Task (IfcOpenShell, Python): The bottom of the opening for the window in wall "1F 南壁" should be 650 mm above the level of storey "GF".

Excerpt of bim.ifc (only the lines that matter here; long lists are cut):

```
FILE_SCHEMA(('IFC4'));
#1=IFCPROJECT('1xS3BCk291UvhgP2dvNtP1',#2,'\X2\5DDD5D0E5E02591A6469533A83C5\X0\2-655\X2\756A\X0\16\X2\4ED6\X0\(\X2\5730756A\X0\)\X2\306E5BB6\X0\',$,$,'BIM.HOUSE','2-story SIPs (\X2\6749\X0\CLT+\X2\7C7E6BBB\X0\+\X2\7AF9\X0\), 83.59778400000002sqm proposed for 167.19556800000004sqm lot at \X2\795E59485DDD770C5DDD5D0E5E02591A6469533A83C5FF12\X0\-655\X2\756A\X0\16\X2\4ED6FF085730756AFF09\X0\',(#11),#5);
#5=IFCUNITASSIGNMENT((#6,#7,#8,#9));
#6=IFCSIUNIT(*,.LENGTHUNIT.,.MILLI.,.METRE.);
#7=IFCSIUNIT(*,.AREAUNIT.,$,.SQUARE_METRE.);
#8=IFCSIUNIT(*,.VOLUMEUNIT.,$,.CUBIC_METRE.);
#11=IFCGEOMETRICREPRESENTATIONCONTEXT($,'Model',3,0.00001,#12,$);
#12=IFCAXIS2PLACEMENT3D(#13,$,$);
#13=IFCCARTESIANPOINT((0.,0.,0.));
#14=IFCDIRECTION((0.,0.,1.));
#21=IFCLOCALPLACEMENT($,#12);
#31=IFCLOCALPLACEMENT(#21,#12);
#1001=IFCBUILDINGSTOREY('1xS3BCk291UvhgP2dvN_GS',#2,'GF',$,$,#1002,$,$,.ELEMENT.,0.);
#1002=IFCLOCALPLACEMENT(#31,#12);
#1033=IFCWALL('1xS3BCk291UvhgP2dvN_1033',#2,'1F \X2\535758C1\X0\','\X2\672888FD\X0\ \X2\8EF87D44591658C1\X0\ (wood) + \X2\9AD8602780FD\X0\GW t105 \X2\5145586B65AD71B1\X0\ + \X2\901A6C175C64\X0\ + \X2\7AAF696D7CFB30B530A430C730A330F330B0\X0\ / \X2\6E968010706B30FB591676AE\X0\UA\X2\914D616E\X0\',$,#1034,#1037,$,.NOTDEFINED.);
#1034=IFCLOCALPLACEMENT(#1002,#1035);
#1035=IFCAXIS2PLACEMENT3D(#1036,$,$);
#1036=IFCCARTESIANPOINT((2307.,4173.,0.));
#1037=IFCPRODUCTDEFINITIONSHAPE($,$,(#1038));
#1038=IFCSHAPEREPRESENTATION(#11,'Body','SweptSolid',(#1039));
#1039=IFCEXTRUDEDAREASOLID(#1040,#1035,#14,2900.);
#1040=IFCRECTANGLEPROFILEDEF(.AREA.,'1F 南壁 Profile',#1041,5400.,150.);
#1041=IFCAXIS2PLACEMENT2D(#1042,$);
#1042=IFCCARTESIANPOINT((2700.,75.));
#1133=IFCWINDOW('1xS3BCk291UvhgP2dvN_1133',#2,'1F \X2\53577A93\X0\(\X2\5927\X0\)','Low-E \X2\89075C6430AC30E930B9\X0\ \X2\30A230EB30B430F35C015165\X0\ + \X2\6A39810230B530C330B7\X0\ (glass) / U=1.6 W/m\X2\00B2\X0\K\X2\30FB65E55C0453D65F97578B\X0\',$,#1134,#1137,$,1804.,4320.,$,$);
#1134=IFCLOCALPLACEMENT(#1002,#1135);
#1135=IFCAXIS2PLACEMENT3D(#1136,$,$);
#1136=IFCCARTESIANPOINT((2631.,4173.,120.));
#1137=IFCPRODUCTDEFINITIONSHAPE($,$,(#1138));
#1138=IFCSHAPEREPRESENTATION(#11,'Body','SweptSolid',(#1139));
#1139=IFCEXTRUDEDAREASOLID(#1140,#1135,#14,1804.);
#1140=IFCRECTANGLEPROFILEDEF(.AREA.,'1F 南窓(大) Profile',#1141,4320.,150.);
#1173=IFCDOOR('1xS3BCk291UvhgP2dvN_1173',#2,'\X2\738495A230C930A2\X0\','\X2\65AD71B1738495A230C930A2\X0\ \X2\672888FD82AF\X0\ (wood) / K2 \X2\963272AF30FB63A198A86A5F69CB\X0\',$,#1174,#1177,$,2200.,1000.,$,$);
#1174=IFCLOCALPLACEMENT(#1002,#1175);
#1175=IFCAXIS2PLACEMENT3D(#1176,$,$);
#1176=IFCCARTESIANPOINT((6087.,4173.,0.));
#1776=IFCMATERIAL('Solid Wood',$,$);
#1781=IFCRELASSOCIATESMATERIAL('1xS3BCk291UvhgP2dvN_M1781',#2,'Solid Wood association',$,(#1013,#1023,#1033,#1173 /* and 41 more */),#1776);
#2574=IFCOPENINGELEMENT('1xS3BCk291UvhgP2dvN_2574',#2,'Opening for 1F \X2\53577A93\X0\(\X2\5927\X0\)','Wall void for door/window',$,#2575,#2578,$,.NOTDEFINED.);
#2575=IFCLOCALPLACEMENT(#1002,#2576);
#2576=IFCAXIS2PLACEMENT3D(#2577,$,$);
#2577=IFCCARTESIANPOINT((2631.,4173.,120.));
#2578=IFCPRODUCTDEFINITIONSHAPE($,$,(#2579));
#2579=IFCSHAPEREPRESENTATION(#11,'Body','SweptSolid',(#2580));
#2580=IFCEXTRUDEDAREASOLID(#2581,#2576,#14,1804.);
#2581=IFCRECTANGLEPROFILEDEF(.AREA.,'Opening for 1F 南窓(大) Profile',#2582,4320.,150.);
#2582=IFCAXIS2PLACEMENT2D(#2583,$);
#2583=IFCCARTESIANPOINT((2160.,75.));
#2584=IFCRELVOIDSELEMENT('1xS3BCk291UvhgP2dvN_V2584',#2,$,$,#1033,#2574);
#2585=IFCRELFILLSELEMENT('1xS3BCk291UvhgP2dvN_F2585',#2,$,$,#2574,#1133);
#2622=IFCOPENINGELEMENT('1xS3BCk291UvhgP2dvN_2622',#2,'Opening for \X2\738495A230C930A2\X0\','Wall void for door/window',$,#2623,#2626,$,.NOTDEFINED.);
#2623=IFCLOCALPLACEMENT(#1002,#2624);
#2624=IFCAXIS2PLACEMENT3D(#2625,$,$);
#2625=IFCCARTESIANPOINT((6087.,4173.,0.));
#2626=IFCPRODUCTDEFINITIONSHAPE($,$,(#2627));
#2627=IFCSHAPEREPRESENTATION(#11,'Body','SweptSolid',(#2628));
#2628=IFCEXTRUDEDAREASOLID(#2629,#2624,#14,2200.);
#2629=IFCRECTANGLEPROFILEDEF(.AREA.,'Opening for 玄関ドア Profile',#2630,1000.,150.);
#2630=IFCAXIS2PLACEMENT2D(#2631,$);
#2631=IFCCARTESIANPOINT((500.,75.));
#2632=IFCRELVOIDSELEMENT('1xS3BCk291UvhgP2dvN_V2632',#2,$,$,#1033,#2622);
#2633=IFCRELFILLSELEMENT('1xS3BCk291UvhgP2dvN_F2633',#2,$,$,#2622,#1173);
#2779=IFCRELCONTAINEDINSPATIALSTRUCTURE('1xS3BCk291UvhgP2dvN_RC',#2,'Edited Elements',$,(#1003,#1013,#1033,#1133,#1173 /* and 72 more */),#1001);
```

```python
import numpy as np
import ifcopenshell
import ifcopenshell.api.geometry
import ifcopenshell.geom
import ifcopenshell.util.element
import ifcopenshell.util.placement
import ifcopenshell.util.shape
import ifcopenshell.util.unit

model = ifcopenshell.open("bim.ifc")
unit_scale = ifcopenshell.util.unit.calculate_unit_scale(model)

window = model.by_guid("1xS3BCk291UvhgP2dvN_1133")
opening = window.FillsVoids[0].RelatingOpeningElement
storey = ifcopenshell.util.element.get_container(window, ifc_class="IfcBuildingStorey")
level = ifcopenshell.util.placement.get_local_placement(storey.ObjectPlacement)[2, 3]

# The opening's origin need not be at the sill, so measure its lowest point.
shape = ifcopenshell.geom.create_shape(ifcopenshell.geom.settings(), opening)
bottom = ifcopenshell.util.shape.get_shape_bottom_elevation(shape, shape.geometry) / unit_scale
dz = level + 0.65 / unit_scale - bottom

shift = np.array([0.0, 0.0, dz])
# The window is not placed relative to its opening, so move both.
for product in (opening, window):
    matrix = ifcopenshell.util.placement.get_local_placement(product.ObjectPlacement)
    matrix[:3, 3] += shift
    ifcopenshell.api.geometry.edit_object_placement(model, product=product, matrix=matrix, is_si=False)

print(f"moved by {dz * unit_scale:+.3f} m")

model.write("bim_v2.ifc")
```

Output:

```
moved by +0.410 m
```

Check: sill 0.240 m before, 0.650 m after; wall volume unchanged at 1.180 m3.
